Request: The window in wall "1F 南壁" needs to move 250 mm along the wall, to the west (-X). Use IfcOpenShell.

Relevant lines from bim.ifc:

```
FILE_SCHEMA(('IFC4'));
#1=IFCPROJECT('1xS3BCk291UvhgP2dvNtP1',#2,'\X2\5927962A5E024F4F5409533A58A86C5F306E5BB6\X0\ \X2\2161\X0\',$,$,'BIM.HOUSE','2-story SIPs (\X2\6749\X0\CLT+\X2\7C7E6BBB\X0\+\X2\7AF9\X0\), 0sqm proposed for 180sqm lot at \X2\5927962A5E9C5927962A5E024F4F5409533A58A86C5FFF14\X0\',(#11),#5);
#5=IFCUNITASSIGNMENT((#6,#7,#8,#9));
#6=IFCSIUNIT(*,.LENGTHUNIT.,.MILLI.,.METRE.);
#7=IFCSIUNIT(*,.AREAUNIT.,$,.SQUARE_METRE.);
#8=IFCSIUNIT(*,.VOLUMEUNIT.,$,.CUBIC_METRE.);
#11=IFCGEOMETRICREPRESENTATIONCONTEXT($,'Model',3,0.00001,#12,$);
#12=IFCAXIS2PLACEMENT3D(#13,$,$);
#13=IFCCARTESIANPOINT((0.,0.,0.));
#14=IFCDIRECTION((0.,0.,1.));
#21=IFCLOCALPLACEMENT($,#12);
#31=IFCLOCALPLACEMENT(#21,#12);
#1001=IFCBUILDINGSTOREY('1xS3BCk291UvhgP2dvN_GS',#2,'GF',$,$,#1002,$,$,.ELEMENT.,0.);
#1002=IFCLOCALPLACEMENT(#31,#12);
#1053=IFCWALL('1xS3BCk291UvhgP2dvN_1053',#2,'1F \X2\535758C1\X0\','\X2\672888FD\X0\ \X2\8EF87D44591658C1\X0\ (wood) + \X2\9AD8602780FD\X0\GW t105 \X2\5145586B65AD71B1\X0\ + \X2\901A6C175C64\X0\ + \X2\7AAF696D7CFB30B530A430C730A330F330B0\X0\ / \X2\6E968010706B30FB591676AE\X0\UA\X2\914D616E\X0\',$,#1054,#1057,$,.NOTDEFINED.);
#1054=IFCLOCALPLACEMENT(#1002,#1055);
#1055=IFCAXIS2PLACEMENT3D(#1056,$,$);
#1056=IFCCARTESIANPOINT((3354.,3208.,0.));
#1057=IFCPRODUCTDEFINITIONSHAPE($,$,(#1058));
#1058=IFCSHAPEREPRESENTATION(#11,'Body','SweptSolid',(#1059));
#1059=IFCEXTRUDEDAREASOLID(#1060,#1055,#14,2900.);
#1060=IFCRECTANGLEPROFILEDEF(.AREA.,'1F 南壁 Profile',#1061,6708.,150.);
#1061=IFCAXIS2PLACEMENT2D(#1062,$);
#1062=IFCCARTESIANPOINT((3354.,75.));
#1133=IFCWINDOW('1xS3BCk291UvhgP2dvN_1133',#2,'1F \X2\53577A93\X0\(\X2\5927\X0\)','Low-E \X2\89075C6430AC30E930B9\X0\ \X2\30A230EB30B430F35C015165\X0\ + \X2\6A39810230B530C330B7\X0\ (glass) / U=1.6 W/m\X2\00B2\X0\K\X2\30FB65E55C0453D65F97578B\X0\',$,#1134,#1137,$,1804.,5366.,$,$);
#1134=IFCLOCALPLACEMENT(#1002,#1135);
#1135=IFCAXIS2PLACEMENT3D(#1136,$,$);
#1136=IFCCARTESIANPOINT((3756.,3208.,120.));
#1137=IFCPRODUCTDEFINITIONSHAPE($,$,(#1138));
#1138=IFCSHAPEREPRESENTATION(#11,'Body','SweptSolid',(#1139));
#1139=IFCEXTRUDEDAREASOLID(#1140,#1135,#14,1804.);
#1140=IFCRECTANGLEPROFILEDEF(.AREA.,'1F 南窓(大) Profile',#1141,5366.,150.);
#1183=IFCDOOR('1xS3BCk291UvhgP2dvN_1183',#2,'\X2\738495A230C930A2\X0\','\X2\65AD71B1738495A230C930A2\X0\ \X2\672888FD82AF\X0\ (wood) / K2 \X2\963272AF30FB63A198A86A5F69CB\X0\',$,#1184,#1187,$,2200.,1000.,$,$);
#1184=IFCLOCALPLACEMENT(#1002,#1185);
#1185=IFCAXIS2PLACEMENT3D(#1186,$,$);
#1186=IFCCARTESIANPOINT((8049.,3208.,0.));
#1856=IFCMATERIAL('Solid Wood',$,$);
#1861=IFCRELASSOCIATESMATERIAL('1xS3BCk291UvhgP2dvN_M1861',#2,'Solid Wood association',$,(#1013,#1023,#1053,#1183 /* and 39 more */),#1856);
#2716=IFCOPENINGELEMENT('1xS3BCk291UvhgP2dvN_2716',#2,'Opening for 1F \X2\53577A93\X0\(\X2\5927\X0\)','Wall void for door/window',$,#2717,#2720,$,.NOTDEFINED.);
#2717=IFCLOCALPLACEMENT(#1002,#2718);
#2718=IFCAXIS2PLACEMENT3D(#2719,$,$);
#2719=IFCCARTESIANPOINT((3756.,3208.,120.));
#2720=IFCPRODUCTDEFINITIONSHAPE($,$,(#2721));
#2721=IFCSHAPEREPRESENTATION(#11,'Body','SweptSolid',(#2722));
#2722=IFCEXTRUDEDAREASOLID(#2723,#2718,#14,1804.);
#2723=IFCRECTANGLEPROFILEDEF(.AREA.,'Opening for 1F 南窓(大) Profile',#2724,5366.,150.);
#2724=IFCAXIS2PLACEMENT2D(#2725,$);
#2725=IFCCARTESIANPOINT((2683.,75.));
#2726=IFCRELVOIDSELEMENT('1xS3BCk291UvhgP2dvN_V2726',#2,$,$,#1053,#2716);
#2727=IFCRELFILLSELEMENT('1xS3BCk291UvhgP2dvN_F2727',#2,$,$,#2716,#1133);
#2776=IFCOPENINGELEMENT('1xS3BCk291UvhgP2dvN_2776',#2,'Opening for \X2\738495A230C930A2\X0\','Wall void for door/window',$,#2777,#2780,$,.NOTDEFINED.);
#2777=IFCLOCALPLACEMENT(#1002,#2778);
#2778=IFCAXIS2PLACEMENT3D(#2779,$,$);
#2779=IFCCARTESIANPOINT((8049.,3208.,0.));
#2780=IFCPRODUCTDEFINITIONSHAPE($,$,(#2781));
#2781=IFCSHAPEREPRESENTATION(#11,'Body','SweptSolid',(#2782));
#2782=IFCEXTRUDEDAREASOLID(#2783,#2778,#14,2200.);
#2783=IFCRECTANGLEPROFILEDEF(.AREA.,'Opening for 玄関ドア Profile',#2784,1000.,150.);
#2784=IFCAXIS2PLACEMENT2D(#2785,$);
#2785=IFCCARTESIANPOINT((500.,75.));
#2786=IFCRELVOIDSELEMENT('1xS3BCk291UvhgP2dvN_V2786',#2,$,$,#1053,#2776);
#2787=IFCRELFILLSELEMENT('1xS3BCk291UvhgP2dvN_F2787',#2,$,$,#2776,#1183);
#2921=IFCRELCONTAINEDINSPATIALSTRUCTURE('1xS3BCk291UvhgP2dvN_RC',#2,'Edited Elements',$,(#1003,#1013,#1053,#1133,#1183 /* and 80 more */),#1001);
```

```python
import ifcopenshell
import ifcopenshell.api.geometry
import ifcopenshell.util.placement
import ifcopenshell.util.unit

model = ifcopenshell.open("bim.ifc")
unit_scale = ifcopenshell.util.unit.calculate_unit_scale(model)

window = model.by_id(1133)
opening = window.FillsVoids[0].RelatingOpeningElement
wall = opening.VoidsElements[0].RelatingBuildingElement

wall_matrix = ifcopenshell.util.placement.get_local_placement(wall.ObjectPlacement)
shift = wall_matrix[:3, 0] * -0.25 / unit_scale
before = ifcopenshell.util.placement.get_local_placement(window.ObjectPlacement)[:3, 3].copy()

# The window is not placed relative to its opening, so move both.
for product in (opening, window):
    matrix = ifcopenshell.util.placement.get_local_placement(product.ObjectPlacement)
    matrix[:3, 3] += shift
    ifcopenshell.api.geometry.edit_object_placement(model, product=product, matrix=matrix, is_si=False)

after = ifcopenshell.util.placement.get_local_placement(window.ObjectPlacement)[:3, 3]
print("window moved by", (after - before).round(3) + 0.0)

model.write("bim_edited.ifc")
```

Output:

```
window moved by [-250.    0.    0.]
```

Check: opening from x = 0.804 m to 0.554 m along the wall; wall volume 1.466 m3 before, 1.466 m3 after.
